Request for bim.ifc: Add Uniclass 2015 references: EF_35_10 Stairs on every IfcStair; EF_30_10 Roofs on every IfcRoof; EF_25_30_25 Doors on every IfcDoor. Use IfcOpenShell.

First a look at what the model holds.

```python
import ifcopenshell

model = ifcopenshell.open("bim.ifc")
print(model.schema)
print("classifications:", [c.Name for c in model.by_type("IfcClassification")])
for ifc_class in ("IfcDoor", "IfcRoof", "IfcStair", "IfcWall", "IfcWindow"):
    print(ifc_class, len(model.by_type(ifc_class)))
```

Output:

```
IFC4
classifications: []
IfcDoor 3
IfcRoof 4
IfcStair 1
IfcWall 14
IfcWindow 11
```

```python
import ifcopenshell
import ifcopenshell.api.classification

model = ifcopenshell.open("bim.ifc")

system = ifcopenshell.api.classification.add_classification(model, classification="Uniclass 2015")

codes = {
    "IfcStair": ("EF_35_10", "Stairs"),
    "IfcRoof": ("EF_30_10", "Roofs"),
    "IfcDoor": ("EF_25_30_25", "Doors"),
}
for ifc_class, (code, name) in codes.items():
    products = model.by_type(ifc_class)
    ifcopenshell.api.classification.add_reference(
        model, products=products, classification=system, identification=code, name=name
    )
    print(code, len(products))

model.write("bim_rev.ifc")
```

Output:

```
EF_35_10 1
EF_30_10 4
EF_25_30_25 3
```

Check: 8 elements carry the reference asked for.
